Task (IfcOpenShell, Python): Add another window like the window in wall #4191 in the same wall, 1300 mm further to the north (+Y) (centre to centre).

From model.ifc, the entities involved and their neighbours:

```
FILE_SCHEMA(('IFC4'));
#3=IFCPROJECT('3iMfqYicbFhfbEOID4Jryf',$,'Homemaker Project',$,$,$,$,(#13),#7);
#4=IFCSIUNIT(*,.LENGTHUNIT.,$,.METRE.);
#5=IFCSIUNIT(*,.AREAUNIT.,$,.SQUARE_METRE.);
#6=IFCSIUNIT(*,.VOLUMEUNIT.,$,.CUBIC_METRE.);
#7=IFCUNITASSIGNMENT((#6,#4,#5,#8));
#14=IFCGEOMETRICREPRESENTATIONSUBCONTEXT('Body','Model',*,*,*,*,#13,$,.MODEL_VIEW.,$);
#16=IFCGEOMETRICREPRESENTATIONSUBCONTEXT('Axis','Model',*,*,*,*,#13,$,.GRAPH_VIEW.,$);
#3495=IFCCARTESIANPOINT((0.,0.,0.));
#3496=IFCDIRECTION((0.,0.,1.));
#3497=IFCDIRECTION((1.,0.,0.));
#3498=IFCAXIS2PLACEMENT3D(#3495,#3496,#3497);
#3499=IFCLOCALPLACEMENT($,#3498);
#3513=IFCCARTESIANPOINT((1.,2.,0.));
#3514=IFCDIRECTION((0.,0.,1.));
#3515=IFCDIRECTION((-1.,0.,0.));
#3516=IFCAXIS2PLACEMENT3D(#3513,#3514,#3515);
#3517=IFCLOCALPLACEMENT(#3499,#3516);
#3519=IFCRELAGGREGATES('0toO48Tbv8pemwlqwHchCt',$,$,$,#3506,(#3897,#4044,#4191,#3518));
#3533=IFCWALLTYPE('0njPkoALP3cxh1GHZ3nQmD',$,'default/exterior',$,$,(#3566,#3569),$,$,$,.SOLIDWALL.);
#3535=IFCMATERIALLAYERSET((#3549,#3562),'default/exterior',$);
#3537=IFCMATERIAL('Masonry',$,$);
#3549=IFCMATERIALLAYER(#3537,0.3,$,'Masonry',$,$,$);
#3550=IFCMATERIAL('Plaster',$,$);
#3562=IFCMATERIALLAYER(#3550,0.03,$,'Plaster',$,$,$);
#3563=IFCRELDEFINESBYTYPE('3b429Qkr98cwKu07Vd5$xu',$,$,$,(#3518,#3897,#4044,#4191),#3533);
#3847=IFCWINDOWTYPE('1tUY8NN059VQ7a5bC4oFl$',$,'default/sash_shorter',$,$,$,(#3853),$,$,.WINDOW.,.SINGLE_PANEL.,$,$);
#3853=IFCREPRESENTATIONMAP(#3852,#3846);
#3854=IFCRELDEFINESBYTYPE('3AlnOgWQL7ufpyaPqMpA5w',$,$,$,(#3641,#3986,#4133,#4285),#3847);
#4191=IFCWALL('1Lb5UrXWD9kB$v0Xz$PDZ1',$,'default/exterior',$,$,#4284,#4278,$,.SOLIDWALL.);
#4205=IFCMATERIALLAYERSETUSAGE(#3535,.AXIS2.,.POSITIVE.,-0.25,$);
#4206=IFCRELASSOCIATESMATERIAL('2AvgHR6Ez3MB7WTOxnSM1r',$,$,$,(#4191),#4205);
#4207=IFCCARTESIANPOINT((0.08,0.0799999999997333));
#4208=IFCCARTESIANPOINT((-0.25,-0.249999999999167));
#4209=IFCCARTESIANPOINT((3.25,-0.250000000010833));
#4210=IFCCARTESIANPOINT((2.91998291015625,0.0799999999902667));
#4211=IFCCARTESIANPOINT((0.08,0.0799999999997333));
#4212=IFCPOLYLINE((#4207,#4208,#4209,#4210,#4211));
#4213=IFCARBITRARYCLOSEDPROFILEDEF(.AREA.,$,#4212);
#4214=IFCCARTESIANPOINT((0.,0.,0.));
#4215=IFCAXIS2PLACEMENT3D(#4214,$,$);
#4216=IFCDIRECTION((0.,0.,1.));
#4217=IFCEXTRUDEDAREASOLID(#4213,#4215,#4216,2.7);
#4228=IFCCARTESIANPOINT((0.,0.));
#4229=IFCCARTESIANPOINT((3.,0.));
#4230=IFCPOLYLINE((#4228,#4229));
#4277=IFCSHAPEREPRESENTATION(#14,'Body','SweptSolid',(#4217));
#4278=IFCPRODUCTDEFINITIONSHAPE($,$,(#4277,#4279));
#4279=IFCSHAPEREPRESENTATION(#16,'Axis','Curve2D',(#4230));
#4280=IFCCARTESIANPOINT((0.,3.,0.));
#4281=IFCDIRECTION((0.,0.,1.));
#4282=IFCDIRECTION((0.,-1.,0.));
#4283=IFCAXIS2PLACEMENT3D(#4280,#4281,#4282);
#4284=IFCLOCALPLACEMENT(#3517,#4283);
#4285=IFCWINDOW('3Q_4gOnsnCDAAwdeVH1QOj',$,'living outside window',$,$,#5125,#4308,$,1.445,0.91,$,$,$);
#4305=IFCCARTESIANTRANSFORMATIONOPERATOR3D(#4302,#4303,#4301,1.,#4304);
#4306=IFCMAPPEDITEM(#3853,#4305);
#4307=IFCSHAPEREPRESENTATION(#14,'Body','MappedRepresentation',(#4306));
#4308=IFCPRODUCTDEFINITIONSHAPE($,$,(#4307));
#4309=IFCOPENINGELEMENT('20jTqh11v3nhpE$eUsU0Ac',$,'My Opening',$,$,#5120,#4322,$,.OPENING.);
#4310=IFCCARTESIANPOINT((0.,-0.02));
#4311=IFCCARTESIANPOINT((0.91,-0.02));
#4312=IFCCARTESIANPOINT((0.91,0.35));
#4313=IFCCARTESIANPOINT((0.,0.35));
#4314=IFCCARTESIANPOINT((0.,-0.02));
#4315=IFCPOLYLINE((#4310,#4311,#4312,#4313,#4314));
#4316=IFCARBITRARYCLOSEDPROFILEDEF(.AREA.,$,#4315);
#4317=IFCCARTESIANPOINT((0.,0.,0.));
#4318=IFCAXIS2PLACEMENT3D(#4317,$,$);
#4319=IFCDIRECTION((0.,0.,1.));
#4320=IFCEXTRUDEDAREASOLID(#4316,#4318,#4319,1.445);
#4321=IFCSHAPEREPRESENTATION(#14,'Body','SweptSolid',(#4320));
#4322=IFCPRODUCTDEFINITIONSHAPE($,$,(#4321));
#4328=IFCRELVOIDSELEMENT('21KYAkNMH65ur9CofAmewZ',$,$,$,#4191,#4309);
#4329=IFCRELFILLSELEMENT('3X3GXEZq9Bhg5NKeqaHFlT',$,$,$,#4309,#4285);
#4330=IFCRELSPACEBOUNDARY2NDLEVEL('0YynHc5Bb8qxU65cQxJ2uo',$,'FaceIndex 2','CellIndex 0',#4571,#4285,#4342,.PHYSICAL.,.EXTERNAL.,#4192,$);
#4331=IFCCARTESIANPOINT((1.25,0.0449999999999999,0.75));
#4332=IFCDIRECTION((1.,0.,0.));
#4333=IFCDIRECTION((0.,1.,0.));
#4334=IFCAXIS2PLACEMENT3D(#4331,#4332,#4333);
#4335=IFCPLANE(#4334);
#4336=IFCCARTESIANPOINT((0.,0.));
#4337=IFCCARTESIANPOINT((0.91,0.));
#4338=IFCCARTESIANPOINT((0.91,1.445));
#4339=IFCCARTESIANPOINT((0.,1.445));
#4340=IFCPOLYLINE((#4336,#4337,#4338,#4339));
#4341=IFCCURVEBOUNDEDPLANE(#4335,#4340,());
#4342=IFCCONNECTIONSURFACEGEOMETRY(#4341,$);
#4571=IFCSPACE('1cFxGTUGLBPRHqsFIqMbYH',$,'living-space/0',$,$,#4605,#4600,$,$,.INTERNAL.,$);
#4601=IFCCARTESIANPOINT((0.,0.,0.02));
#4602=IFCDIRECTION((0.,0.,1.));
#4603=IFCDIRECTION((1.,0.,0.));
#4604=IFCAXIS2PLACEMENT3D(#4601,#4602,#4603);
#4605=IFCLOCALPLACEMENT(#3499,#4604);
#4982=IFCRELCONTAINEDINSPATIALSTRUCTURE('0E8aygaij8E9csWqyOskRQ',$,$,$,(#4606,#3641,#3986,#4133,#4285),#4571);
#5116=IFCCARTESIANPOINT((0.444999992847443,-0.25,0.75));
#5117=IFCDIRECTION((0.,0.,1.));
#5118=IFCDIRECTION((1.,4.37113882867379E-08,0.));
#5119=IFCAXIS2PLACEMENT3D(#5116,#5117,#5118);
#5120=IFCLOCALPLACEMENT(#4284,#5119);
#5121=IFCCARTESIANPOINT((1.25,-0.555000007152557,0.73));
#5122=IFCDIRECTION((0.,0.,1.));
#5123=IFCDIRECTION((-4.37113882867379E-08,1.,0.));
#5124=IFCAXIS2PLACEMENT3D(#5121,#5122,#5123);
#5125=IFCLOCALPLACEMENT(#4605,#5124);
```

```python
import numpy as np
import ifcopenshell
import ifcopenshell.api.feature
import ifcopenshell.api.geometry
import ifcopenshell.api.root
import ifcopenshell.geom
import ifcopenshell.util.element
import ifcopenshell.util.placement
import ifcopenshell.util.shape
import ifcopenshell.util.unit

model = ifcopenshell.open("model.ifc")
unit_scale = ifcopenshell.util.unit.calculate_unit_scale(model)
settings = ifcopenshell.geom.settings()


def volume(element):
    """Net volume in cubic metres, openings subtracted."""
    shape = ifcopenshell.geom.create_shape(settings, element)
    return ifcopenshell.util.shape.get_volume(shape.geometry)


window = model.by_guid("3Q_4gOnsnCDAAwdeVH1QOj")
opening = window.FillsVoids[0].RelatingOpeningElement
wall = opening.VoidsElements[0].RelatingBuildingElement
before = volume(wall)
shift = ifcopenshell.util.placement.get_local_placement(wall.ObjectPlacement)[:3, 0] * 1.3 / unit_scale

# copy_class copies the void relationship, type, container and properties, but no geometry.
new_opening = ifcopenshell.api.root.copy_class(model, product=opening)
new_opening.Representation = ifcopenshell.util.element.copy_deep(
    model, opening.Representation, exclude=["IfcGeometricRepresentationContext", "IfcRepresentationMap"]
)
new_window = ifcopenshell.api.root.copy_class(model, product=window)
new_window.Representation = ifcopenshell.util.element.copy_deep(
    model, window.Representation, exclude=["IfcGeometricRepresentationContext", "IfcRepresentationMap"]
)
ifcopenshell.api.feature.add_filling(model, opening=new_opening, element=new_window)

for old, new in ((opening, new_opening), (window, new_window)):
    matrix = ifcopenshell.util.placement.get_local_placement(old.ObjectPlacement)
    matrix[:3, 3] += shift
    ifcopenshell.api.geometry.edit_object_placement(model, product=new, matrix=matrix, is_si=False)

# The copied space boundaries still share their surfaces with the original.
for rel in new_window.ProvidesBoundaries:
    if rel.ConnectionGeometry:
        rel.ConnectionGeometry = ifcopenshell.util.element.copy_deep(model, rel.ConnectionGeometry)

# Space boundary surfaces are stored in each space's coordinates; move them too.
for rel in new_window.ProvidesBoundaries:
    if not rel.ConnectionGeometry:
        continue
    surface = rel.ConnectionGeometry.SurfaceOnRelatingElement.BasisSurface
    space_matrix = ifcopenshell.util.placement.get_local_placement(rel.RelatingSpace.ObjectPlacement)
    point = np.array(surface.Position.Location.Coordinates) + space_matrix[:3, :3].T @ shift
    surface.Position = model.createIfcAxis2Placement3D(
        model.createIfcCartesianPoint(point.tolist()), surface.Position.Axis, surface.Position.RefDirection
    )

after = volume(wall)

print(f"wall volume {before:.3f} -> {after:.3f} m3")

model.write("model_edited.ifc")
```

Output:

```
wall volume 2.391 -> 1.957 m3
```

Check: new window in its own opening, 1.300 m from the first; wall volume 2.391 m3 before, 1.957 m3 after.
